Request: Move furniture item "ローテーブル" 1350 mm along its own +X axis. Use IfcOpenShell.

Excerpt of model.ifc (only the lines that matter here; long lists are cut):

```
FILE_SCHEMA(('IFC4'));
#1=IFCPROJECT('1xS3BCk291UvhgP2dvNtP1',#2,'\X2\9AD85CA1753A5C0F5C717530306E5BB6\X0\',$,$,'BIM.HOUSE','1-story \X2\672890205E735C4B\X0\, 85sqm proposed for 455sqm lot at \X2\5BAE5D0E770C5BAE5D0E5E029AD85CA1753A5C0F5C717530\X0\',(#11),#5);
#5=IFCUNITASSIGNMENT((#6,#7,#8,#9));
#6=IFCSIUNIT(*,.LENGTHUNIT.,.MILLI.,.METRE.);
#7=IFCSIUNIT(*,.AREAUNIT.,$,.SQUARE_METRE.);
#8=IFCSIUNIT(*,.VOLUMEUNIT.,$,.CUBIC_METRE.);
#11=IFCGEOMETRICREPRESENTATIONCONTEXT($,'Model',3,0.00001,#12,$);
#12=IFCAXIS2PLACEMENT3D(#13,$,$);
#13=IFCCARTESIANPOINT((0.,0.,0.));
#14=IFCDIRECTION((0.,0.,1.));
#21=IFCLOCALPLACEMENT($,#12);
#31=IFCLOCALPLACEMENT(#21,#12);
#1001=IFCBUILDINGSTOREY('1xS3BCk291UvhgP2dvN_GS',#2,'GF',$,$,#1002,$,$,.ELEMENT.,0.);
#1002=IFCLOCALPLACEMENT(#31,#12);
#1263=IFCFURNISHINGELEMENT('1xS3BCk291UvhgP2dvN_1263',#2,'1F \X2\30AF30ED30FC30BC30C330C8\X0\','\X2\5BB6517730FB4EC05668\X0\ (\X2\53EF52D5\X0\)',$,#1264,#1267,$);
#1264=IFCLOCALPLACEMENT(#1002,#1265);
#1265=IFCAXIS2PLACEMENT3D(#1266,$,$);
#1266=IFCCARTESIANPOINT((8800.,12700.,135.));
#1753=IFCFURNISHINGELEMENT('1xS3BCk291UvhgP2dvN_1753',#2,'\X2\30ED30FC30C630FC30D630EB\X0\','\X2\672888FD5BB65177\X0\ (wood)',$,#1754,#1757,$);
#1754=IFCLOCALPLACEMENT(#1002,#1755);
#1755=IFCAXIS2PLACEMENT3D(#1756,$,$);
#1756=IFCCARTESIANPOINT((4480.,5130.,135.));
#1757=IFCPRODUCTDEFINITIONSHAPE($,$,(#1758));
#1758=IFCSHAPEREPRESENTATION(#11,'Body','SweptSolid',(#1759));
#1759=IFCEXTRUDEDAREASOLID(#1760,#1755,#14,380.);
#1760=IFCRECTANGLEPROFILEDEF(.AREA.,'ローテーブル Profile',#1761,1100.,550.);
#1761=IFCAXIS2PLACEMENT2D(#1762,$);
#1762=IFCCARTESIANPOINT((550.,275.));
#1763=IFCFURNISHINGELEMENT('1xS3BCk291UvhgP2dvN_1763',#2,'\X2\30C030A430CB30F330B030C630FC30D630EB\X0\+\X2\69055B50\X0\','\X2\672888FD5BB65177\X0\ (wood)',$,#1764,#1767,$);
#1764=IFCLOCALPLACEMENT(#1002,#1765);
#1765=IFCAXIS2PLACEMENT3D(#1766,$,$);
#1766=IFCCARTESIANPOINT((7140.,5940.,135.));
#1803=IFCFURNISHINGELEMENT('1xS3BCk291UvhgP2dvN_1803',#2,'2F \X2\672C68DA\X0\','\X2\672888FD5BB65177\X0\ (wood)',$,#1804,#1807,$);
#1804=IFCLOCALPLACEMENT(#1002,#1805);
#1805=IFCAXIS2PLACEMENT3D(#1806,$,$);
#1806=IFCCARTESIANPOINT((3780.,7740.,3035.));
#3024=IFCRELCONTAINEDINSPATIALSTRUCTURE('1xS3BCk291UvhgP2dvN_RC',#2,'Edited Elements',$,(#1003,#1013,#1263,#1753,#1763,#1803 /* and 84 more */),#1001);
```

```python
import ifcopenshell
import ifcopenshell.api.geometry
import ifcopenshell.util.placement
import ifcopenshell.util.unit

model = ifcopenshell.open("model.ifc")
unit_scale = ifcopenshell.util.unit.calculate_unit_scale(model)

item = model.by_guid("1xS3BCk291UvhgP2dvN_1753")
matrix = ifcopenshell.util.placement.get_local_placement(item.ObjectPlacement)
matrix[:3, 3] += matrix[:3, 0] * 1.35 / unit_scale
ifcopenshell.api.geometry.edit_object_placement(model, product=item, matrix=matrix, is_si=False)

print(ifcopenshell.util.placement.get_local_placement(item.ObjectPlacement).round(3) + 0.0)

model.write("model_rev.ifc")
```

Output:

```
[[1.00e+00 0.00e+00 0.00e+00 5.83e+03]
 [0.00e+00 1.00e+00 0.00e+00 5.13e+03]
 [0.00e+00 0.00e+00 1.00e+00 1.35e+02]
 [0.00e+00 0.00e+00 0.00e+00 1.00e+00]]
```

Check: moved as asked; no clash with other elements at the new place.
